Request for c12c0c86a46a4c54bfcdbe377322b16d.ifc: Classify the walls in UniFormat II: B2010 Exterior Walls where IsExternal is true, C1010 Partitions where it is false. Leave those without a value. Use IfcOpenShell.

First a look at what the model holds.

```python
import ifcopenshell
import ifcopenshell.util.element

model = ifcopenshell.open("c12c0c86a46a4c54bfcdbe377322b16d.ifc")
print(model.schema)
print("classifications:", [c.Name for c in model.by_type("IfcClassification")])
values = [ifcopenshell.util.element.get_pset(e, "Pset_WallCommon", "IsExternal") for e in model.by_type("IfcWall")]
for value in (True, False, None):
    print("IsExternal", value, values.count(value))
```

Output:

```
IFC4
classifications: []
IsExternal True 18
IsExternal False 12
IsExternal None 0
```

```python
import ifcopenshell
import ifcopenshell.api.classification
import ifcopenshell.util.element

model = ifcopenshell.open("c12c0c86a46a4c54bfcdbe377322b16d.ifc")

system = ifcopenshell.api.classification.add_classification(model, classification="UniFormat II")

walls = model.by_type("IfcWall")
external = {e: ifcopenshell.util.element.get_pset(e, "Pset_WallCommon", "IsExternal") for e in walls}
for flag, code, name in ((True, "B2010", "Exterior Walls"), (False, "C1010", "Partitions")):
    products = [e for e in walls if external[e] is flag]
    ifcopenshell.api.classification.add_reference(
        model, products=products, classification=system, identification=code, name=name
    )
    print(code, len(products))

model.write("c12c0c86a46a4c54bfcdbe377322b16d_rev.ifc")
```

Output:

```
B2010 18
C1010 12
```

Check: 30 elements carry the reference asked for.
